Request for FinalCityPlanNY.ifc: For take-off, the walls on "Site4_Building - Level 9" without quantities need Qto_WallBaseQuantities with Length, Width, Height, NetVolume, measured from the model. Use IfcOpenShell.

First a look at what the model holds.

```python
import ifcopenshell
import ifcopenshell.util.element
import ifcopenshell.util.unit

model = ifcopenshell.open("FinalCityPlanNY.ifc")
print(model.schema)
for unit_type in ("LENGTHUNIT", "AREAUNIT", "VOLUMEUNIT"):
    print(unit_type, ifcopenshell.util.unit.calculate_unit_scale(model, unit_type))
storey = next(s for s in model.by_type("IfcBuildingStorey") if s.Name == "Site4_Building - Level 9")
walls = [e for e in ifcopenshell.util.element.get_decomposition(storey) if e.is_a("IfcWall")]
for e in sorted(walls, key=lambda e: e.id()):
    print(e.id(), e.is_a(), e.Name, list(ifcopenshell.util.element.get_psets(e, qtos_only=True)), sep=" | ")
```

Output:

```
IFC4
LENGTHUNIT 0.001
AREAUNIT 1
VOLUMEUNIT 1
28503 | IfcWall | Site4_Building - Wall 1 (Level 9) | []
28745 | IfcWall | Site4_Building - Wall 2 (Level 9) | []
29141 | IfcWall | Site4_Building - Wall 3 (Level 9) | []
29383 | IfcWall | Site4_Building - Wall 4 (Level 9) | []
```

```python
import ifcopenshell
import ifcopenshell.api.pset
import ifcopenshell.geom
import ifcopenshell.util.element
import ifcopenshell.util.shape
import ifcopenshell.util.unit

model = ifcopenshell.open("FinalCityPlanNY.ifc")
unit_scale = ifcopenshell.util.unit.calculate_unit_scale(model)
volume_scale = ifcopenshell.util.unit.calculate_unit_scale(model, "VOLUMEUNIT")
settings = ifcopenshell.geom.settings()

storey = next(s for s in model.by_type("IfcBuildingStorey") if s.Name == "Site4_Building - Level 9")
walls = [e for e in ifcopenshell.util.element.get_decomposition(storey) if e.is_a("IfcWall")]

for e in sorted(walls, key=lambda e: e.id()):
    if ifcopenshell.util.element.get_psets(e, qtos_only=True, should_inherit=False):
        continue
    # Geometry comes back in metres, in the element's own axes.
    shape = ifcopenshell.geom.create_shape(settings, e)
    values = {
        "Length": ifcopenshell.util.shape.get_x(shape.geometry) / unit_scale,
        "Width": ifcopenshell.util.shape.get_y(shape.geometry) / unit_scale,
        "Height": ifcopenshell.util.shape.get_z(shape.geometry) / unit_scale,
        "NetVolume": ifcopenshell.util.shape.get_volume(shape.geometry) / volume_scale,
    }
    qto = ifcopenshell.api.pset.add_qto(model, product=e, name="Qto_WallBaseQuantities")
    ifcopenshell.api.pset.edit_qto(model, qto=qto, properties=values)
    print(e.id(), {k: round(v, 3) for k, v in values.items()})

model.write("FinalCityPlanNY_rev.ifc")
```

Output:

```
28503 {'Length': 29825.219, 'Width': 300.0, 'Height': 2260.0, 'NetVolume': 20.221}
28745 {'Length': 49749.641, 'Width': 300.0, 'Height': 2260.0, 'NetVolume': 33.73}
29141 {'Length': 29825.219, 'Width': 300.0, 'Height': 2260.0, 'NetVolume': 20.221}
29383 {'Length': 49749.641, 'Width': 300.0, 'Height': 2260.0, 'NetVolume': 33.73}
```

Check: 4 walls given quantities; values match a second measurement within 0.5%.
